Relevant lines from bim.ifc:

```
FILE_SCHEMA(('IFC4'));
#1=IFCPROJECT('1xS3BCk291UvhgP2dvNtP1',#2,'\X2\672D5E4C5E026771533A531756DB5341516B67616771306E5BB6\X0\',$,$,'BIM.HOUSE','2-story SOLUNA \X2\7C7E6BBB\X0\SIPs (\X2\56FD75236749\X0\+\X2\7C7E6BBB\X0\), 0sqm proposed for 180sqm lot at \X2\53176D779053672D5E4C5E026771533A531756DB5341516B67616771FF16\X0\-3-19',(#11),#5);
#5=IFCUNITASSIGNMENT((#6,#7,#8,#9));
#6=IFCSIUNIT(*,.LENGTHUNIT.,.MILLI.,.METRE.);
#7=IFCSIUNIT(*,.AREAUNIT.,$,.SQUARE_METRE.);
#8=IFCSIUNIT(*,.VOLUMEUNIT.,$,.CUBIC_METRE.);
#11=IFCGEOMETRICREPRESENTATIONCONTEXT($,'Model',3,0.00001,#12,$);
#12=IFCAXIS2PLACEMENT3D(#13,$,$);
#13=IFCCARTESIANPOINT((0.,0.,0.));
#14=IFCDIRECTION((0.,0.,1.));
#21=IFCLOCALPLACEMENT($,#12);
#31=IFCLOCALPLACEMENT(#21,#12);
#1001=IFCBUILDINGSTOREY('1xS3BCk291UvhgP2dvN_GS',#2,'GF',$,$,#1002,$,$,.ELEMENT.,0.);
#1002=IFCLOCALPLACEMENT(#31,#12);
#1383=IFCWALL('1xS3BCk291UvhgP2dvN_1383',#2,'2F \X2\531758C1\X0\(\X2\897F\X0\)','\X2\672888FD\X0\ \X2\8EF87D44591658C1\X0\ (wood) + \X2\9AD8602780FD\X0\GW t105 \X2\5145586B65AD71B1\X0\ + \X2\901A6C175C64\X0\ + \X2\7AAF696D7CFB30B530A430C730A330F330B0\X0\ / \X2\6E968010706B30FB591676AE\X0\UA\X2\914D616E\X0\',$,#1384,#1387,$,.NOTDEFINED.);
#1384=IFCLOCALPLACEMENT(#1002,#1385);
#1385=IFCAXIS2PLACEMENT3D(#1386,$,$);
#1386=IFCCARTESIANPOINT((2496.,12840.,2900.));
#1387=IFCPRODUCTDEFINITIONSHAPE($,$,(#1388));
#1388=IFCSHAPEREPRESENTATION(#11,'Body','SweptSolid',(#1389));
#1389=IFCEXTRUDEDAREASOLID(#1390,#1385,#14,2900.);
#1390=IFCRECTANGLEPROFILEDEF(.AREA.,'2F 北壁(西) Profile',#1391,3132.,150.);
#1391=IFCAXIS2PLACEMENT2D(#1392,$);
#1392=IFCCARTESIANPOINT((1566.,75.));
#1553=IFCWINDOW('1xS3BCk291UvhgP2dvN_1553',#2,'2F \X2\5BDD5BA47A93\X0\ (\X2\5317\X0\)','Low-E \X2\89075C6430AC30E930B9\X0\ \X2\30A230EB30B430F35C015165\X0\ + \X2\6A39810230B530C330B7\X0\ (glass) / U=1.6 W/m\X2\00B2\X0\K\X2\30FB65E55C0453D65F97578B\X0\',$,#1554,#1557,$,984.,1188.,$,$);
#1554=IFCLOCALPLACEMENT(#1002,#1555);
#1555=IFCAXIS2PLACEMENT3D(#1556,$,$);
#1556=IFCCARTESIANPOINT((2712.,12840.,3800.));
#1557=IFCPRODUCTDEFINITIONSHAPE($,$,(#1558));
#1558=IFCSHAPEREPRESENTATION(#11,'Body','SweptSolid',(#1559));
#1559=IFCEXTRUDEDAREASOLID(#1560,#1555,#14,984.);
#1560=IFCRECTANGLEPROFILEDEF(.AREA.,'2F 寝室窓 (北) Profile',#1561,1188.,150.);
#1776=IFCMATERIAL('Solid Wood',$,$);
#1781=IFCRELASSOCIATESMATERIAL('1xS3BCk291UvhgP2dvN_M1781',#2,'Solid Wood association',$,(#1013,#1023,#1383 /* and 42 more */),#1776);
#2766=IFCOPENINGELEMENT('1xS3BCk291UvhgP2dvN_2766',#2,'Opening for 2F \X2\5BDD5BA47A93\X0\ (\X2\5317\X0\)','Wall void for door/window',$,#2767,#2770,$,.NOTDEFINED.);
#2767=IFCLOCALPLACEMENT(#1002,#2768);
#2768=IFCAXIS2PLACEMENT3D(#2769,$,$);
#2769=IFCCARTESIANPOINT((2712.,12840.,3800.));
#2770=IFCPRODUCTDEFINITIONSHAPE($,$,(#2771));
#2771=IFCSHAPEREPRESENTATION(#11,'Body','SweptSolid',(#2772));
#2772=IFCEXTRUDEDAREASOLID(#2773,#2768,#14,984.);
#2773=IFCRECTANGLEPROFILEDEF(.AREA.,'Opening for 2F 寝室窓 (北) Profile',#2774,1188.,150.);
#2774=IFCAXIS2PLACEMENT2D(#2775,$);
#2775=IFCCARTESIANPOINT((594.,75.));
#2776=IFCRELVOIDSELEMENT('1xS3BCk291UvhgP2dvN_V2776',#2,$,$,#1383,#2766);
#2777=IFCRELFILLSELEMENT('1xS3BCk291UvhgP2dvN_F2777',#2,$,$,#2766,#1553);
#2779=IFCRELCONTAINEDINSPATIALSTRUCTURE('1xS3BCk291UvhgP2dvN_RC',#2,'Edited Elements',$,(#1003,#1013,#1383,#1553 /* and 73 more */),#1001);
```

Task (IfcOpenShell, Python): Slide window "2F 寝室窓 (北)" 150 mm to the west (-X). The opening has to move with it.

```python
import ifcopenshell
import ifcopenshell.api.geometry
import ifcopenshell.util.placement

model = ifcopenshell.open("bim.ifc")

window = model.by_guid("1xS3BCk291UvhgP2dvN_1553")
opening = window.FillsVoids[0].RelatingOpeningElement
wall = opening.VoidsElements[0].RelatingBuildingElement

wall_matrix = ifcopenshell.util.placement.get_local_placement(wall.ObjectPlacement)
shift = wall_matrix[:3, 0] * -150.0
before = ifcopenshell.util.placement.get_local_placement(window.ObjectPlacement)[:3, 3].copy()

# The window is not placed relative to its opening, so move both.
for product in (opening, window):
    matrix = ifcopenshell.util.placement.get_local_placement(product.ObjectPlacement)
    matrix[:3, 3] += shift
    ifcopenshell.api.geometry.edit_object_placement(model, product=product, matrix=matrix, is_si=False)

after = ifcopenshell.util.placement.get_local_placement(window.ObjectPlacement)[:3, 3]
print("window moved by", (after - before).round(3) + 0.0)

model.write("bim_edited.ifc")
```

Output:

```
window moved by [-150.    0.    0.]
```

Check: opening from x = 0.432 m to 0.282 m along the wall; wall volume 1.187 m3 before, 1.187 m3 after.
